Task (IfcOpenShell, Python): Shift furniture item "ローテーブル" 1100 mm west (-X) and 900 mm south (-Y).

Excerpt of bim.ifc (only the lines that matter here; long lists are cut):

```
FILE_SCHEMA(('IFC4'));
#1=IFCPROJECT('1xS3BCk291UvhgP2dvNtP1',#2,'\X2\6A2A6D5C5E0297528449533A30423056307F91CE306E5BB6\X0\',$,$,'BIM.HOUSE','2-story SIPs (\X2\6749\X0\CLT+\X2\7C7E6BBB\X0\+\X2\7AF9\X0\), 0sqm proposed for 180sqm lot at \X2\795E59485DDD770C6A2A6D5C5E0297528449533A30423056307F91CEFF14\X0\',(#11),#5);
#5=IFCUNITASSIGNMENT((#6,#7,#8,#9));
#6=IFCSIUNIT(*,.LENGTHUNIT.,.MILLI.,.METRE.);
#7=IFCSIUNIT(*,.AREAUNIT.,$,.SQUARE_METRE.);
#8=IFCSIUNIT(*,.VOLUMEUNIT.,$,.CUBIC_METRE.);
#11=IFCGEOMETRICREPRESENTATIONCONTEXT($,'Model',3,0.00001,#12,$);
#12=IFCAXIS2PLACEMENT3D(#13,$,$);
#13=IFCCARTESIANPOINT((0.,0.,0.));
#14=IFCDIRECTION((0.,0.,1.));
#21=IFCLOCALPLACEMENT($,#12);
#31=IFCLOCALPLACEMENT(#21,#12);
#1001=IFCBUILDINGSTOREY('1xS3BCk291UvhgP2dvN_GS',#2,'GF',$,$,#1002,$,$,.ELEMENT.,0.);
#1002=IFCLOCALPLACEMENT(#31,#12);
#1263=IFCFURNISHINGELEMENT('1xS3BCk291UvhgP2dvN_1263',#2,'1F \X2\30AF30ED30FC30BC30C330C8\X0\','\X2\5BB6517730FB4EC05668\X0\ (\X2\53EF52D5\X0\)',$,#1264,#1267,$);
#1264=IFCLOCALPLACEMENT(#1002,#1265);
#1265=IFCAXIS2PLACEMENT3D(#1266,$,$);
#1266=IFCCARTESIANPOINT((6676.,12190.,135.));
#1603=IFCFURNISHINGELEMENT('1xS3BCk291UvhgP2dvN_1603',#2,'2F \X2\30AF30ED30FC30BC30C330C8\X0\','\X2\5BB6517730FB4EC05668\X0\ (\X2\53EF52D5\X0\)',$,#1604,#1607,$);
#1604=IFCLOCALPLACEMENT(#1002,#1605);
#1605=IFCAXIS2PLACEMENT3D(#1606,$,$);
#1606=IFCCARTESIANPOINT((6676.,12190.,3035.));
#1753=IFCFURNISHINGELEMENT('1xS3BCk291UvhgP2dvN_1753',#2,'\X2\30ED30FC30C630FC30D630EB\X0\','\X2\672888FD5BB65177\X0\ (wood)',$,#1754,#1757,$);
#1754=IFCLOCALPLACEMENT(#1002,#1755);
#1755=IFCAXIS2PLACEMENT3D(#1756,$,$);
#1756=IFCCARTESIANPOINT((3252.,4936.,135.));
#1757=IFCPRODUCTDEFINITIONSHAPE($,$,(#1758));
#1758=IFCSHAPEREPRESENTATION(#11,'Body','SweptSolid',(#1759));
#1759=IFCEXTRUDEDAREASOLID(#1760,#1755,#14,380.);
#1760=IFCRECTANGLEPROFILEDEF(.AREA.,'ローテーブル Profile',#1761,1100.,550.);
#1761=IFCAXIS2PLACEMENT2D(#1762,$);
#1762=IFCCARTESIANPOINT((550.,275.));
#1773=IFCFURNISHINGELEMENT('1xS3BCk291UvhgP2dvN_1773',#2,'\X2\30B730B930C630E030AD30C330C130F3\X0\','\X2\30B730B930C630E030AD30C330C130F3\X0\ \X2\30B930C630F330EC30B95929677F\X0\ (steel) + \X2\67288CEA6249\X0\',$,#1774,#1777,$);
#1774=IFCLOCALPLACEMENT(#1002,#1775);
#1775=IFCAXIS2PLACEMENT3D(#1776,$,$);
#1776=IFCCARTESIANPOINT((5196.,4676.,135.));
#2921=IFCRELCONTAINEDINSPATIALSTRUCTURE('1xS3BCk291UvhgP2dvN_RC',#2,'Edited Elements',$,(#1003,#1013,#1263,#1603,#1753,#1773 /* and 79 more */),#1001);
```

```python
import ifcopenshell
import ifcopenshell.api.geometry
import ifcopenshell.util.placement

model = ifcopenshell.open("bim.ifc")

item = model.by_guid("1xS3BCk291UvhgP2dvN_1753")
matrix = ifcopenshell.util.placement.get_local_placement(item.ObjectPlacement)
matrix[0, 3] -= 1100.0
matrix[1, 3] -= 900.0
ifcopenshell.api.geometry.edit_object_placement(model, product=item, matrix=matrix, is_si=False)

print(ifcopenshell.util.placement.get_local_placement(item.ObjectPlacement).round(3) + 0.0)

model.write("bim_v2.ifc")
```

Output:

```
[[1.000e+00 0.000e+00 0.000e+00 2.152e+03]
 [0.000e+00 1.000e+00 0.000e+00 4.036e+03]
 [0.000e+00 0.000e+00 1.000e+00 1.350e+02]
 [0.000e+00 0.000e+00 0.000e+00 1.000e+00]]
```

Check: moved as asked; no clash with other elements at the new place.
